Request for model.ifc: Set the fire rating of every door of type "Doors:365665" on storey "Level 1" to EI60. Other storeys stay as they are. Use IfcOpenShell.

First a look at what the model holds.

```python
import ifcopenshell
import ifcopenshell.util.element

model = ifcopenshell.open("model.ifc")
print(model.schema)
storey = next(s for s in model.by_type("IfcBuildingStorey") if s.Name == "Level 1")
doors = [e for e in ifcopenshell.util.element.get_decomposition(storey) if e.is_a("IfcDoor")]
seen = {}
for e in doors:
    element_type = ifcopenshell.util.element.get_type(e)
    key = (element_type.Name if element_type != e and element_type else None, ifcopenshell.util.element.get_pset(e, "Pset_DoorCommon", "FireRating"))
    seen[key] = seen.get(key, 0) + 1
for (name, value), count in sorted(seen.items(), key=str):
    print(count, "x", name, "|", value)
```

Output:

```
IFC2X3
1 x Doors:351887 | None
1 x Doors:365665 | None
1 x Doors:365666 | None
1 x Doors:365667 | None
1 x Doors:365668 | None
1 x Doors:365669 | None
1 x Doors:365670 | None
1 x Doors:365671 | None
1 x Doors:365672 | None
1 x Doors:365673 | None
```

```python
import ifcopenshell
import ifcopenshell.api.pset
import ifcopenshell.util.element

model = ifcopenshell.open("model.ifc")

storey = next(s for s in model.by_type("IfcBuildingStorey") if s.Name == "Level 1")
doors = [e for e in ifcopenshell.util.element.get_decomposition(storey) if e.is_a("IfcDoor")]

count = 0
for e in doors:
    element_type = ifcopenshell.util.element.get_type(e)
    if element_type in (None, e) or element_type.Name != "Doors:365665":
        continue
    # add_pset returns the element's existing set when there is one.
    pset = ifcopenshell.api.pset.add_pset(model, product=e, name="Pset_DoorCommon")
    ifcopenshell.api.pset.edit_pset(model, pset=pset, properties={"FireRating": "EI60"})
    count += 1

print(count, "doors updated")

model.write("model_v2.ifc")
```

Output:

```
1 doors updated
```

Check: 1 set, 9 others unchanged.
